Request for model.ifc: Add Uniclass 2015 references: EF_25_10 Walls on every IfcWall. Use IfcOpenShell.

First a look at what the model holds.

```python
import ifcopenshell

model = ifcopenshell.open("model.ifc")
print(model.schema)
print("classifications:", [c.Name for c in model.by_type("IfcClassification")])
for ifc_class in ("IfcDoor", "IfcRoof", "IfcStair", "IfcWall", "IfcWindow"):
    print(ifc_class, len(model.by_type(ifc_class)))
```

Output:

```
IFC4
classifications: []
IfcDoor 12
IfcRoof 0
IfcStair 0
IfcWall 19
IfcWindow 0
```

```python
import ifcopenshell
import ifcopenshell.api.classification

model = ifcopenshell.open("model.ifc")

system = ifcopenshell.api.classification.add_classification(model, classification="Uniclass 2015")

codes = {
    "IfcWall": ("EF_25_10", "Walls"),
}
for ifc_class, (code, name) in codes.items():
    products = model.by_type(ifc_class)
    ifcopenshell.api.classification.add_reference(
        model, products=products, classification=system, identification=code, name=name
    )
    print(code, len(products))

model.write("model_edited.ifc")
```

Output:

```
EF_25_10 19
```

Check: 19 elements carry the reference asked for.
